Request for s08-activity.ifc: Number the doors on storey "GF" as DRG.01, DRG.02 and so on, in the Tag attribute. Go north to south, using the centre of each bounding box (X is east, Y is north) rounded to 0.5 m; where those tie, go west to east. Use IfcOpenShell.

First a look at what the model holds.

```python
import ifcopenshell
import ifcopenshell.util.element
import ifcopenshell.util.placement

model = ifcopenshell.open("s08-activity.ifc")
print(model.schema)
storey = next(s for s in model.by_type("IfcBuildingStorey") if s.Name == "GF")
doors = [e for e in ifcopenshell.util.element.get_decomposition(storey) if e.is_a("IfcDoor")]
for e in sorted(doors, key=lambda e: e.id()):
    origin = ifcopenshell.util.placement.get_local_placement(e.ObjectPlacement)[:3, 3]
    print(e.id(), e.Tag, e.Name, origin.round(2) + 0.0, sep=" | ")
```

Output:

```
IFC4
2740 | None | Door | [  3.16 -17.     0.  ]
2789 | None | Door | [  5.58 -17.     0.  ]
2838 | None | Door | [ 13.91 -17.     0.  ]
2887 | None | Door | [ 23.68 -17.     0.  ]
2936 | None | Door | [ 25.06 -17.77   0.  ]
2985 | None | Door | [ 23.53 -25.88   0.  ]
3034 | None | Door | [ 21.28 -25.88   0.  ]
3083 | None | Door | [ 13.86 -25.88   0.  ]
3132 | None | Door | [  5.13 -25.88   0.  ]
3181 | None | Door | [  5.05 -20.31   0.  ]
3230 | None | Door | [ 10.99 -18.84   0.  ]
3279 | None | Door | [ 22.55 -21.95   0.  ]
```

```python
import ifcopenshell
import ifcopenshell.geom
import ifcopenshell.util.element
import ifcopenshell.util.shape

model = ifcopenshell.open("s08-activity.ifc")
settings = ifcopenshell.geom.settings()
settings.set("use-world-coords", True)


def centre(element):
    shape = ifcopenshell.geom.create_shape(settings, element)
    return ifcopenshell.util.shape.get_bbox_centroid(shape.geometry)


storey = next(s for s in model.by_type("IfcBuildingStorey") if s.Name == "GF")
doors = [e for e in ifcopenshell.util.element.get_decomposition(storey) if e.is_a("IfcDoor")]

# Insertion points can sit at a corner or the storey origin, so sort by the geometry (in metres).
centres = {e: centre(e) for e in doors}
doors.sort(key=lambda e: (-round(centres[e][1] / 0.5), centres[e][0]))

for i, e in enumerate(doors, start=1):
    number = f"DRG.{i:02d}"
    e.Tag = number
    print(e.id(), number)

model.write("s08-activity_v2.ifc")
```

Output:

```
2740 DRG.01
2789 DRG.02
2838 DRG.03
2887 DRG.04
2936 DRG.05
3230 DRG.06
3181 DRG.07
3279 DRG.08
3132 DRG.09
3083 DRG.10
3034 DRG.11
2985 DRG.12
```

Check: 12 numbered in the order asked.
